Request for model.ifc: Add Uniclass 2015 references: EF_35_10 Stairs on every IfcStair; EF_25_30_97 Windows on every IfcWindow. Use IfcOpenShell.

First a look at what the model holds.

```python
import ifcopenshell

model = ifcopenshell.open("model.ifc")
print(model.schema)
print("classifications:", [c.Name for c in model.by_type("IfcClassification")])
for ifc_class in ("IfcDoor", "IfcRoof", "IfcStair", "IfcWall", "IfcWindow"):
    print(ifc_class, len(model.by_type(ifc_class)))
```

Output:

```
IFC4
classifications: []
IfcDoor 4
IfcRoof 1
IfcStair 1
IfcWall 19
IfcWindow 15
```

```python
import ifcopenshell
import ifcopenshell.api.classification

model = ifcopenshell.open("model.ifc")

system = ifcopenshell.api.classification.add_classification(model, classification="Uniclass 2015")

codes = {
    "IfcStair": ("EF_35_10", "Stairs"),
    "IfcWindow": ("EF_25_30_97", "Windows"),
}
for ifc_class, (code, name) in codes.items():
    products = model.by_type(ifc_class)
    ifcopenshell.api.classification.add_reference(
        model, products=products, classification=system, identification=code, name=name
    )
    print(code, len(products))

model.write("model_updated.ifc")
```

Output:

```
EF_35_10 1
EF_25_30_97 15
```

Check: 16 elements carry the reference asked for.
